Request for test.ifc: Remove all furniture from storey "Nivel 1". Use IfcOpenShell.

First a look at what the model holds.

```python
import ifcopenshell
import ifcopenshell.util.element

model = ifcopenshell.open("test.ifc")
print(model.schema)
storey = next(s for s in model.by_type("IfcBuildingStorey") if s.Name == "Nivel 1")
furniture = [e for e in ifcopenshell.util.element.get_decomposition(storey) if e.is_a("IfcFurnishingElement")]
seen = {}
for e in furniture:
    element_type = ifcopenshell.util.element.get_type(e)
    name = element_type.Name if element_type not in (None, e) else None
    seen[name] = seen.get(name, 0) + 1
for name, count in sorted(seen.items(), key=str):
    print(count, "x", name)
```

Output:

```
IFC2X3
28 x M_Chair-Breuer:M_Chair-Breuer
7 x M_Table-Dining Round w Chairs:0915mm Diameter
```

```python
import ifcopenshell
import ifcopenshell.api.root
import ifcopenshell.util.element

model = ifcopenshell.open("test.ifc")

storey = next(s for s in model.by_type("IfcBuildingStorey") if s.Name == "Nivel 1")
furniture = [e for e in ifcopenshell.util.element.get_decomposition(storey) if e.is_a("IfcFurnishingElement")]

for e in furniture:
    ifcopenshell.api.root.remove_product(model, product=e)
print(len(furniture), "removed")

model.write("test_v2.ifc")
```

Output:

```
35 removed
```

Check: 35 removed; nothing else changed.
